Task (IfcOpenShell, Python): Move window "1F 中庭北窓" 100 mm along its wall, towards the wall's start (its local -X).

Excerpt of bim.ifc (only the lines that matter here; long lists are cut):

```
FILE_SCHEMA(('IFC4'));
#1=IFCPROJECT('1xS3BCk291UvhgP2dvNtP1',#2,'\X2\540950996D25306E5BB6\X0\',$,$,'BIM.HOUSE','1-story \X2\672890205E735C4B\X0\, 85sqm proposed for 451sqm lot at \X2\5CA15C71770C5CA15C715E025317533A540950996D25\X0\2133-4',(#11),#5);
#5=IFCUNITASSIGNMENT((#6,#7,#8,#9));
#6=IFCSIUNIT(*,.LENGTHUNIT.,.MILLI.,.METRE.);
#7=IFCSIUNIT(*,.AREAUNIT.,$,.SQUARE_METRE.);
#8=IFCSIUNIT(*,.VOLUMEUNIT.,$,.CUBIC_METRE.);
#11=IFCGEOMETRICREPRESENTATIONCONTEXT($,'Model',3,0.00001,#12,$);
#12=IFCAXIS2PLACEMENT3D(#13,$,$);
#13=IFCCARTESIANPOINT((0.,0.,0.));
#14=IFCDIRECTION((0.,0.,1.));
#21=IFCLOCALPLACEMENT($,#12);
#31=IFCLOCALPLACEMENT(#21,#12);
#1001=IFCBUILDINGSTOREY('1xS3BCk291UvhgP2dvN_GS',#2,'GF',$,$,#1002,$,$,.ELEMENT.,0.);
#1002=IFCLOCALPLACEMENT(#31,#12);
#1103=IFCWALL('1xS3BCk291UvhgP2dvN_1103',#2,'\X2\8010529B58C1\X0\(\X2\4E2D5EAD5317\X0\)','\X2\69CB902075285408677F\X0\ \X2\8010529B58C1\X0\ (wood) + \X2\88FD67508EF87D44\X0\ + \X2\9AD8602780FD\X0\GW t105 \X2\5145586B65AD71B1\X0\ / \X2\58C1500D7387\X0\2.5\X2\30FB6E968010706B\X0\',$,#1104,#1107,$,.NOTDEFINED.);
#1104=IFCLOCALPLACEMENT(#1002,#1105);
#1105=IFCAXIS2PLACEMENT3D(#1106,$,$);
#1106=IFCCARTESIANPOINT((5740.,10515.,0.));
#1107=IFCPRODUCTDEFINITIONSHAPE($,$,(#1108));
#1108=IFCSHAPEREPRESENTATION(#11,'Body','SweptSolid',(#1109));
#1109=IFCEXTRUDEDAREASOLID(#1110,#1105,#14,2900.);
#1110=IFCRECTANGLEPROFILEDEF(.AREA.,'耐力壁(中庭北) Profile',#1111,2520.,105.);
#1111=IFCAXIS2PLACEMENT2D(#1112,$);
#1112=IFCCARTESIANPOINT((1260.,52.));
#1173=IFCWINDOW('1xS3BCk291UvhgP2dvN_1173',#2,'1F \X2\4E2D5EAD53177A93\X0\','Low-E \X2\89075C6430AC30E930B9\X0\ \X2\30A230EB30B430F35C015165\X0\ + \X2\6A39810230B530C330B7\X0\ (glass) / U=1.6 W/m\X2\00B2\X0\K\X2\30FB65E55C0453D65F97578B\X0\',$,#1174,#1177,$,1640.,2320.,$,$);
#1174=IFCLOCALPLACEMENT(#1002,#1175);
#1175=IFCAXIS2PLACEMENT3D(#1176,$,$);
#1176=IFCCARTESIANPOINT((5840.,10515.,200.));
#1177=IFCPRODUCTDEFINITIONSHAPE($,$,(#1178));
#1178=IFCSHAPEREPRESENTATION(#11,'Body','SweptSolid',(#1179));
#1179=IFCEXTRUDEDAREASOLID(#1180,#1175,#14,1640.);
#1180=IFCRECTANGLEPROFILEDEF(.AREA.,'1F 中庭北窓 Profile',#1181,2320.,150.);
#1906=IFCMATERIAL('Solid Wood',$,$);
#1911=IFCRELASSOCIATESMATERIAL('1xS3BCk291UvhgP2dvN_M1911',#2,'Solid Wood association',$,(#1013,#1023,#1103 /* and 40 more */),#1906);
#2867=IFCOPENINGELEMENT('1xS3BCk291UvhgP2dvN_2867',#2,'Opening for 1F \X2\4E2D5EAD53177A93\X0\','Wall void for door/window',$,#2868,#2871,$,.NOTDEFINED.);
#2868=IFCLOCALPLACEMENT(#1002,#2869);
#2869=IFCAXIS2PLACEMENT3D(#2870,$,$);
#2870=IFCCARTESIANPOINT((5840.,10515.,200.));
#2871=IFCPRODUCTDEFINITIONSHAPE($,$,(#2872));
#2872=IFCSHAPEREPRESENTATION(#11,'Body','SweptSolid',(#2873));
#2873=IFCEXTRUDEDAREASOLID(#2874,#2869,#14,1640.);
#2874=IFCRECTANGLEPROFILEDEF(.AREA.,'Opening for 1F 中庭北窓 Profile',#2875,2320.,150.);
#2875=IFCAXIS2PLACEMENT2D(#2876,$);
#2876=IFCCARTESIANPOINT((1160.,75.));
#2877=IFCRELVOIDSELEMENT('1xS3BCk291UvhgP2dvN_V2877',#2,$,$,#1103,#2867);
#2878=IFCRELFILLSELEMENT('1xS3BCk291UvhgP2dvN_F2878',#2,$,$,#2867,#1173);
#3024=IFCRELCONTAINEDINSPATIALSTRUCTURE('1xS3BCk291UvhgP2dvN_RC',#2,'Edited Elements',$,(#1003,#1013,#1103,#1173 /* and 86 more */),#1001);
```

```python
import ifcopenshell
import ifcopenshell.api.geometry
import ifcopenshell.util.placement
import ifcopenshell.util.unit

model = ifcopenshell.open("bim.ifc")
unit_scale = ifcopenshell.util.unit.calculate_unit_scale(model)

window = model.by_guid("1xS3BCk291UvhgP2dvN_1173")
opening = window.FillsVoids[0].RelatingOpeningElement
wall = opening.VoidsElements[0].RelatingBuildingElement

wall_matrix = ifcopenshell.util.placement.get_local_placement(wall.ObjectPlacement)
shift = wall_matrix[:3, 0] * -0.1 / unit_scale
before = ifcopenshell.util.placement.get_local_placement(window.ObjectPlacement)[:3, 3].copy()

# The window is not placed relative to its opening, so move both.
for product in (opening, window):
    matrix = ifcopenshell.util.placement.get_local_placement(product.ObjectPlacement)
    matrix[:3, 3] += shift
    ifcopenshell.api.geometry.edit_object_placement(model, product=product, matrix=matrix, is_si=False)

after = ifcopenshell.util.placement.get_local_placement(window.ObjectPlacement)[:3, 3]
print("window moved by", (after - before).round(3) + 0.0)

model.write("bim-out.ifc")
```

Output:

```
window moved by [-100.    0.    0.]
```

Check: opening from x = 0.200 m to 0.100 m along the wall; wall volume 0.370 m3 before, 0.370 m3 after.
